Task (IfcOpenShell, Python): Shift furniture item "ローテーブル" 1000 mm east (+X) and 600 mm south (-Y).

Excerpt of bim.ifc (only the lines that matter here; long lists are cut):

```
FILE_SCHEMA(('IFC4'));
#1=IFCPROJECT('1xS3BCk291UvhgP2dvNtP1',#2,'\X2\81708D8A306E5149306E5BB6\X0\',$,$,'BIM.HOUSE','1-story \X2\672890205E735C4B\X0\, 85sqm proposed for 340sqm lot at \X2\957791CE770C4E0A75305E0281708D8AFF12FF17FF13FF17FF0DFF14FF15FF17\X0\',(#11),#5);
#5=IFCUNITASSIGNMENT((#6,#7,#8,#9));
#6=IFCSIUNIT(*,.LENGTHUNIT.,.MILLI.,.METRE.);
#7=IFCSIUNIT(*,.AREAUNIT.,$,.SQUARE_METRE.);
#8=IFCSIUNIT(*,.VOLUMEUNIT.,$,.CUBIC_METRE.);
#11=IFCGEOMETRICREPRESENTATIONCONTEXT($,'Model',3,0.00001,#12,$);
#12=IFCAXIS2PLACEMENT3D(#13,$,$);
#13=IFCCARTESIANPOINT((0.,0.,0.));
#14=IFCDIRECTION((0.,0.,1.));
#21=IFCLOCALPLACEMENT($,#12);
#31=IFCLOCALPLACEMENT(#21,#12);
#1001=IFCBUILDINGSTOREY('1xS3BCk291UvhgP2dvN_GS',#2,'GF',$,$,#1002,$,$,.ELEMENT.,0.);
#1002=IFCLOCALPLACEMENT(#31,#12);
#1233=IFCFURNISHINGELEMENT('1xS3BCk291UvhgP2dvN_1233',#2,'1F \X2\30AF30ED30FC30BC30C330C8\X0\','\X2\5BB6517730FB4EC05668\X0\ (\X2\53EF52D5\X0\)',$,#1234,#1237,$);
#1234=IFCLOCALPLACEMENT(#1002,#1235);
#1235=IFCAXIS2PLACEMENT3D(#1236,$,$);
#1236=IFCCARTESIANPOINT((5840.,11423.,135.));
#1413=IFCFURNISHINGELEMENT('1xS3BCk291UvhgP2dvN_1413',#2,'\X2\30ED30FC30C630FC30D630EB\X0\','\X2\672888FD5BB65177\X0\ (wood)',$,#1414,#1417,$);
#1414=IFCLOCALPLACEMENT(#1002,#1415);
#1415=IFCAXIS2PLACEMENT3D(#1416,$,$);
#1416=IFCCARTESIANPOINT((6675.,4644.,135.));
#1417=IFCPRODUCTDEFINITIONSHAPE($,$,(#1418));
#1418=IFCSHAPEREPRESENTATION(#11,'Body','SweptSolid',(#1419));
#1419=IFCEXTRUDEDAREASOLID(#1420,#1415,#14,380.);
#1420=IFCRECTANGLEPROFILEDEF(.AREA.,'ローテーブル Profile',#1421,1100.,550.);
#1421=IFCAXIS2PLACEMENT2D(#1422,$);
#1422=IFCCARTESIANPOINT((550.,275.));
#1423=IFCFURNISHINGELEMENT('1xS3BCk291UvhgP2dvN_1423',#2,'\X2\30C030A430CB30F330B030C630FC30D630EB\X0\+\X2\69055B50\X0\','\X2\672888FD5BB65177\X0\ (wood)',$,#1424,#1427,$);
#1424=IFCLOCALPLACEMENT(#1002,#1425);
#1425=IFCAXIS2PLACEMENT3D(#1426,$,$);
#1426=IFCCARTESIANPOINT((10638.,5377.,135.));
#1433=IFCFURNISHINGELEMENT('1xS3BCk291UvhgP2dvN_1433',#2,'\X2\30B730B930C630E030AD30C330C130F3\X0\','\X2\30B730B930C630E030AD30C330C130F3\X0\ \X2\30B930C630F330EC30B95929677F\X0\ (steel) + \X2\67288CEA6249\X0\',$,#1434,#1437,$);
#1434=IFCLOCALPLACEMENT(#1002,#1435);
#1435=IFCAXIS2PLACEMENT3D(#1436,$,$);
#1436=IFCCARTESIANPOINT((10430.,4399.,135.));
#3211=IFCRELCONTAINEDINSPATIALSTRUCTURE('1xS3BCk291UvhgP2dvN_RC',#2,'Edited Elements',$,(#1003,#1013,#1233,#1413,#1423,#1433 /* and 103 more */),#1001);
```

```python
import ifcopenshell
import ifcopenshell.api.geometry
import ifcopenshell.util.placement

model = ifcopenshell.open("bim.ifc")

item = model.by_guid("1xS3BCk291UvhgP2dvN_1413")
matrix = ifcopenshell.util.placement.get_local_placement(item.ObjectPlacement)
matrix[0, 3] += 1000.0
matrix[1, 3] -= 600.0
ifcopenshell.api.geometry.edit_object_placement(model, product=item, matrix=matrix, is_si=False)

print(ifcopenshell.util.placement.get_local_placement(item.ObjectPlacement).round(3) + 0.0)

model.write("bim_rev.ifc")
```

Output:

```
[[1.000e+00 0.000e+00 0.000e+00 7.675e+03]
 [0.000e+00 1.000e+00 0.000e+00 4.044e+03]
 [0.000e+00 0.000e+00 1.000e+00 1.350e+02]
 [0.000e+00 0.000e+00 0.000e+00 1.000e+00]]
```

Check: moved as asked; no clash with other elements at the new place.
